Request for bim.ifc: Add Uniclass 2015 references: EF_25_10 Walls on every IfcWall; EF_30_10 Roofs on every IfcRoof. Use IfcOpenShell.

First a look at what the model holds.

```python
import ifcopenshell

model = ifcopenshell.open("bim.ifc")
print(model.schema)
print("classifications:", [c.Name for c in model.by_type("IfcClassification")])
for ifc_class in ("IfcDoor", "IfcRoof", "IfcStair", "IfcWall", "IfcWindow"):
    print(ifc_class, len(model.by_type(ifc_class)))
```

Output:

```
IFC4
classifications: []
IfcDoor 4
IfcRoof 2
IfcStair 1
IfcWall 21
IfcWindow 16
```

```python
import ifcopenshell
import ifcopenshell.api.classification

model = ifcopenshell.open("bim.ifc")

system = ifcopenshell.api.classification.add_classification(model, classification="Uniclass 2015")

codes = {
    "IfcWall": ("EF_25_10", "Walls"),
    "IfcRoof": ("EF_30_10", "Roofs"),
}
for ifc_class, (code, name) in codes.items():
    products = model.by_type(ifc_class)
    ifcopenshell.api.classification.add_reference(
        model, products=products, classification=system, identification=code, name=name
    )
    print(code, len(products))

model.write("bim_rev.ifc")
```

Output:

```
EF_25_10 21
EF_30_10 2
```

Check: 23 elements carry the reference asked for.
